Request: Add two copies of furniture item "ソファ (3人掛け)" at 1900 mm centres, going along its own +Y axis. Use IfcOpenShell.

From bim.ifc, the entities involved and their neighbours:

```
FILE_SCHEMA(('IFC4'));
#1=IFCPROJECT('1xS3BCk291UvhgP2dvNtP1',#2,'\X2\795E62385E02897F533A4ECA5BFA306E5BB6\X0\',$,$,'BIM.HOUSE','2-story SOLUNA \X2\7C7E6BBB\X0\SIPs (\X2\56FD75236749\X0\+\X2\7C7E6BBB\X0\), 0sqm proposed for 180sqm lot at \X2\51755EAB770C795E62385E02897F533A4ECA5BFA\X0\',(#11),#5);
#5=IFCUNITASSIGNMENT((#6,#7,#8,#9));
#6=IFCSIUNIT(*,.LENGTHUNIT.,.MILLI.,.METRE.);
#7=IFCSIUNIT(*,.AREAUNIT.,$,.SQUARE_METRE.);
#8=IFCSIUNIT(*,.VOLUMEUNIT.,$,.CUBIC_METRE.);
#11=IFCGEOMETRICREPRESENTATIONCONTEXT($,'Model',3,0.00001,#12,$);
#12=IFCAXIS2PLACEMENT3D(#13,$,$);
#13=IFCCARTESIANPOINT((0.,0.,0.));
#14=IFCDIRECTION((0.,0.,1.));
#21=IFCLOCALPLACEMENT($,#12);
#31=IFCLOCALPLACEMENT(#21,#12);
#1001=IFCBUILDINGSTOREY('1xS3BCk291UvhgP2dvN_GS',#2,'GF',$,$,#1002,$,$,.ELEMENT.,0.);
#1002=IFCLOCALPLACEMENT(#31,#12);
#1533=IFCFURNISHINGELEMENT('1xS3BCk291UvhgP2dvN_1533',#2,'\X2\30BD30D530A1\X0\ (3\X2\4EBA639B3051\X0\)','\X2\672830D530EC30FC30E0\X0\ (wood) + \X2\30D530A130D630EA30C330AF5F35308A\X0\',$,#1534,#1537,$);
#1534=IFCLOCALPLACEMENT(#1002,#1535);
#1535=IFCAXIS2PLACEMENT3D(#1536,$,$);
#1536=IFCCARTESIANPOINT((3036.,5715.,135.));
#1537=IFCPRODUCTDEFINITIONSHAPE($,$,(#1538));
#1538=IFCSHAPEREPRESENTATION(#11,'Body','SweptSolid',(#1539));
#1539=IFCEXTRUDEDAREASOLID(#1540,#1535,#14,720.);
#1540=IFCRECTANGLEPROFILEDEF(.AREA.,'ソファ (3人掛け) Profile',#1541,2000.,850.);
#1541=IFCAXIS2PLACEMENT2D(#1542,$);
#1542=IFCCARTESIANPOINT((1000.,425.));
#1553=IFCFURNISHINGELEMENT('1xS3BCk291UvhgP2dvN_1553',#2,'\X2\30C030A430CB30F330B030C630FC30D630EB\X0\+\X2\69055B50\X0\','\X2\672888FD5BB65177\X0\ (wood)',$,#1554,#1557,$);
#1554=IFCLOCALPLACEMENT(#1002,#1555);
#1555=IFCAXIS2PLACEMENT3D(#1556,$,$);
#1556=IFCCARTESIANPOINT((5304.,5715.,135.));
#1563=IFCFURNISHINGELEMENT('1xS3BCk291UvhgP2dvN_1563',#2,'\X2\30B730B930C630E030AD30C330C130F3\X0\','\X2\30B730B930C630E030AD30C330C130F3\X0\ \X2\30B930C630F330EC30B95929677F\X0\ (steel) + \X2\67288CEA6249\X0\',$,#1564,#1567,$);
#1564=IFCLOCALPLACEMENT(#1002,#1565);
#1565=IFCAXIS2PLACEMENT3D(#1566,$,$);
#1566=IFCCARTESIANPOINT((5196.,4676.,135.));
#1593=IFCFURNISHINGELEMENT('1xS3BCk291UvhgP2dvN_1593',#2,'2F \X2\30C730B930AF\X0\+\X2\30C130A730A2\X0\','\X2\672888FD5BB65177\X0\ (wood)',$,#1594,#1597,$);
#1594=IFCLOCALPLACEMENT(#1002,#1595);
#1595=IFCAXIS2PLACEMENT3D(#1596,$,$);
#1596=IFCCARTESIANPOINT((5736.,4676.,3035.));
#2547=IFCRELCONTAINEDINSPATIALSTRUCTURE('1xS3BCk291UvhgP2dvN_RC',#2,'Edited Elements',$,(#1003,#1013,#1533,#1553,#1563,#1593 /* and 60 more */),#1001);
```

```python
import ifcopenshell
import ifcopenshell.api.geometry
import ifcopenshell.api.root
import ifcopenshell.util.element
import ifcopenshell.util.placement

model = ifcopenshell.open("bim.ifc")


def reuse_history(source, copy):
    """copy_class also copies each property set's owner history, people and application; keep the originals."""
    for rel in copy.IsDefinedBy:
        if rel.is_a("IfcRelDefinesByProperties") and (history := rel.RelatingPropertyDefinition.OwnerHistory):
            rel.RelatingPropertyDefinition.OwnerHistory = source.OwnerHistory
            ifcopenshell.util.element.remove_deep2(model, history)


source = model.by_guid("1xS3BCk291UvhgP2dvN_1533")
base = ifcopenshell.util.placement.get_local_placement(source.ObjectPlacement)
step = base[:3, 1] * 1900.0

for i in range(1, 3):
    copy = ifcopenshell.api.root.copy_class(model, product=source)
    copy.Representation = ifcopenshell.util.element.copy_deep(
        model, source.Representation, exclude=["IfcGeometricRepresentationContext", "IfcRepresentationMap"]
    )
    reuse_history(source, copy)
    matrix = base.copy()
    matrix[:3, 3] += i * step
    print("added at", matrix[:3, 3].round(3) + 0.0)
    ifcopenshell.api.geometry.edit_object_placement(model, product=copy, matrix=matrix, is_si=False)

model.write("bim_updated.ifc")
```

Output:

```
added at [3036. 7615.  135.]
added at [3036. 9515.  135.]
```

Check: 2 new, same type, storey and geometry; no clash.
